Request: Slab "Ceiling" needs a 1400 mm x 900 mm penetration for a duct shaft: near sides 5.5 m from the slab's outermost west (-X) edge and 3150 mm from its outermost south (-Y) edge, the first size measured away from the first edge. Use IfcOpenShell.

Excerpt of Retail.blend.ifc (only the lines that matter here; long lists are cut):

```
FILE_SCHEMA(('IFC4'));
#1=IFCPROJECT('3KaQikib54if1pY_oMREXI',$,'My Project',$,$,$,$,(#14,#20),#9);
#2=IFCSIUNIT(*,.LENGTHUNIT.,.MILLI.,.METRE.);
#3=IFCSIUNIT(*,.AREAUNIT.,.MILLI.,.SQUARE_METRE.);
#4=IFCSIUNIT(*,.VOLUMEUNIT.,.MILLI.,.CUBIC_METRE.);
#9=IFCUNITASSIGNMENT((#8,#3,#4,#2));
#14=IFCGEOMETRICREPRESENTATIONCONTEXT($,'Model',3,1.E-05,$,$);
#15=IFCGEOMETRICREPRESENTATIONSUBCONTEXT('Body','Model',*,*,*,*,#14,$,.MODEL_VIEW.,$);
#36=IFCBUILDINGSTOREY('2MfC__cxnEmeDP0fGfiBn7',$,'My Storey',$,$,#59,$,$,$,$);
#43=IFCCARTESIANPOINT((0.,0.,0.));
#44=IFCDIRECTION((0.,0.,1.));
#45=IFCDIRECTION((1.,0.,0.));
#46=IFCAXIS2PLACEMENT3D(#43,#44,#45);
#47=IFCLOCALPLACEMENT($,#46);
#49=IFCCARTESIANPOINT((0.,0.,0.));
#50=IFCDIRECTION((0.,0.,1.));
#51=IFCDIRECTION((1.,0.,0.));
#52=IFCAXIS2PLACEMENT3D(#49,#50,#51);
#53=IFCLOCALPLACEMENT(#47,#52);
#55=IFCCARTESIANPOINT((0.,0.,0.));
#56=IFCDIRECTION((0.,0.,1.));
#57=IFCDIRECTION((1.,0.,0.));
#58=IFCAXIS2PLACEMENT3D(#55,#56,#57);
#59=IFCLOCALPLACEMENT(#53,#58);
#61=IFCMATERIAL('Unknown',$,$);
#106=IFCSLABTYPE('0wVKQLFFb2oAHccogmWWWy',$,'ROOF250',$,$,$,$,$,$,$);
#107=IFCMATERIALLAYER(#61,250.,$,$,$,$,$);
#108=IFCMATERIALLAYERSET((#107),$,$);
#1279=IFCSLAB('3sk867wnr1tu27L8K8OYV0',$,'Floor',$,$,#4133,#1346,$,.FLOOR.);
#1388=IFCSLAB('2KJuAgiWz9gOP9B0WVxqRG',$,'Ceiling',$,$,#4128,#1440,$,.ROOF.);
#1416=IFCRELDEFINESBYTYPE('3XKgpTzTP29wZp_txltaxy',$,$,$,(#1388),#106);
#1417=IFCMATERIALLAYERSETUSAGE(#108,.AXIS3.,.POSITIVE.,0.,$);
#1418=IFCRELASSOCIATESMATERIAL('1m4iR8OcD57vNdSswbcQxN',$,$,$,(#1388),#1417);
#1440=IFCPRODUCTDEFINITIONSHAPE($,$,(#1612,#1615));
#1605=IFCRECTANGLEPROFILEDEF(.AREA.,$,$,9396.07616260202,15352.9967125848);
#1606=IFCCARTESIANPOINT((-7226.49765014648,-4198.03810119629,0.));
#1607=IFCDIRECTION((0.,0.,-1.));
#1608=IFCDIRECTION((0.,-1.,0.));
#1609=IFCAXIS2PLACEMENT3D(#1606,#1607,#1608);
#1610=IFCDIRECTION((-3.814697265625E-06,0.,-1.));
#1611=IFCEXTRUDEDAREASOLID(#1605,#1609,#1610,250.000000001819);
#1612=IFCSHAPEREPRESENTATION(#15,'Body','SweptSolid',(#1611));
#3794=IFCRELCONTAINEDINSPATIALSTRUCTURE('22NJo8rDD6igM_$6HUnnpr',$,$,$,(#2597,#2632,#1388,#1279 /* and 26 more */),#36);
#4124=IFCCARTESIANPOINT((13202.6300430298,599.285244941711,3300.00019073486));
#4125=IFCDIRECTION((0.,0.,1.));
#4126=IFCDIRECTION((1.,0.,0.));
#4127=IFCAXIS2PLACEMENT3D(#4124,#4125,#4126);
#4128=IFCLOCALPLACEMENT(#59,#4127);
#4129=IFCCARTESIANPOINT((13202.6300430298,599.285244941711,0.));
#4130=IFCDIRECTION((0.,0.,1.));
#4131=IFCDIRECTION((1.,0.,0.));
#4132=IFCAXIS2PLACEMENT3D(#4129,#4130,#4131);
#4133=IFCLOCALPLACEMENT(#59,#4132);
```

```python
import numpy as np
import ifcopenshell
import ifcopenshell.api.feature
import ifcopenshell.api.geometry
import ifcopenshell.api.root
import ifcopenshell.geom
import ifcopenshell.util.placement
import ifcopenshell.util.representation
import ifcopenshell.util.shape
import ifcopenshell.util.unit

model = ifcopenshell.open("Retail.blend.ifc")
unit_scale = ifcopenshell.util.unit.calculate_unit_scale(model)
settings = ifcopenshell.geom.settings()


def volume(element):
    """Net volume in cubic metres, openings subtracted."""
    shape = ifcopenshell.geom.create_shape(settings, element)
    return ifcopenshell.util.shape.get_volume(shape.geometry)


slab = model.by_guid("2KJuAgiWz9gOP9B0WVxqRG")
before = volume(slab)

# Extent in the slab's own axes, in metres. The edges named are its -X and -Y sides.
slab_shape = ifcopenshell.geom.create_shape(settings, slab)
vertices = ifcopenshell.util.shape.get_vertices(slab_shape.geometry)
x_min, y_min, bottom = vertices.min(axis=0)
top = vertices[:, 2].max()

opening = ifcopenshell.api.root.create_entity(model, ifc_class="IfcOpeningElement", name="Duct shaft opening", predefined_type="OPENING")
context = ifcopenshell.util.representation.get_context(model, "Model", "Body", "MODEL_VIEW")
width, depth = 1.4, 0.9
outline = [(0.0, 0.0), (width, 0.0), (width, depth), (0.0, depth), (0.0, 0.0)]
# Overshoot both faces by 50 mm so the cut is clean.
shape = ifcopenshell.api.geometry.add_slab_representation(
    model, context=context, depth=top - bottom + 0.1, polyline=outline
)
ifcopenshell.api.geometry.assign_representation(model, product=opening, representation=shape)

matrix = ifcopenshell.util.placement.get_local_placement(slab.ObjectPlacement)
matrix[:, 3] = matrix @ np.append(np.array([x_min + 5.5, y_min + 3.15, bottom - 0.05]) / unit_scale, 1.0)
ifcopenshell.api.geometry.edit_object_placement(model, product=opening, matrix=matrix, is_si=False)
ifcopenshell.api.feature.add_feature(model, feature=opening, element=slab)

after = volume(slab)

print(f"slab volume {before:.3f} -> {after:.3f} m3")

model.write("Retail.blend_updated.ifc")
```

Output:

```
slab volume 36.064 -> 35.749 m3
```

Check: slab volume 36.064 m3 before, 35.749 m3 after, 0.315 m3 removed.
